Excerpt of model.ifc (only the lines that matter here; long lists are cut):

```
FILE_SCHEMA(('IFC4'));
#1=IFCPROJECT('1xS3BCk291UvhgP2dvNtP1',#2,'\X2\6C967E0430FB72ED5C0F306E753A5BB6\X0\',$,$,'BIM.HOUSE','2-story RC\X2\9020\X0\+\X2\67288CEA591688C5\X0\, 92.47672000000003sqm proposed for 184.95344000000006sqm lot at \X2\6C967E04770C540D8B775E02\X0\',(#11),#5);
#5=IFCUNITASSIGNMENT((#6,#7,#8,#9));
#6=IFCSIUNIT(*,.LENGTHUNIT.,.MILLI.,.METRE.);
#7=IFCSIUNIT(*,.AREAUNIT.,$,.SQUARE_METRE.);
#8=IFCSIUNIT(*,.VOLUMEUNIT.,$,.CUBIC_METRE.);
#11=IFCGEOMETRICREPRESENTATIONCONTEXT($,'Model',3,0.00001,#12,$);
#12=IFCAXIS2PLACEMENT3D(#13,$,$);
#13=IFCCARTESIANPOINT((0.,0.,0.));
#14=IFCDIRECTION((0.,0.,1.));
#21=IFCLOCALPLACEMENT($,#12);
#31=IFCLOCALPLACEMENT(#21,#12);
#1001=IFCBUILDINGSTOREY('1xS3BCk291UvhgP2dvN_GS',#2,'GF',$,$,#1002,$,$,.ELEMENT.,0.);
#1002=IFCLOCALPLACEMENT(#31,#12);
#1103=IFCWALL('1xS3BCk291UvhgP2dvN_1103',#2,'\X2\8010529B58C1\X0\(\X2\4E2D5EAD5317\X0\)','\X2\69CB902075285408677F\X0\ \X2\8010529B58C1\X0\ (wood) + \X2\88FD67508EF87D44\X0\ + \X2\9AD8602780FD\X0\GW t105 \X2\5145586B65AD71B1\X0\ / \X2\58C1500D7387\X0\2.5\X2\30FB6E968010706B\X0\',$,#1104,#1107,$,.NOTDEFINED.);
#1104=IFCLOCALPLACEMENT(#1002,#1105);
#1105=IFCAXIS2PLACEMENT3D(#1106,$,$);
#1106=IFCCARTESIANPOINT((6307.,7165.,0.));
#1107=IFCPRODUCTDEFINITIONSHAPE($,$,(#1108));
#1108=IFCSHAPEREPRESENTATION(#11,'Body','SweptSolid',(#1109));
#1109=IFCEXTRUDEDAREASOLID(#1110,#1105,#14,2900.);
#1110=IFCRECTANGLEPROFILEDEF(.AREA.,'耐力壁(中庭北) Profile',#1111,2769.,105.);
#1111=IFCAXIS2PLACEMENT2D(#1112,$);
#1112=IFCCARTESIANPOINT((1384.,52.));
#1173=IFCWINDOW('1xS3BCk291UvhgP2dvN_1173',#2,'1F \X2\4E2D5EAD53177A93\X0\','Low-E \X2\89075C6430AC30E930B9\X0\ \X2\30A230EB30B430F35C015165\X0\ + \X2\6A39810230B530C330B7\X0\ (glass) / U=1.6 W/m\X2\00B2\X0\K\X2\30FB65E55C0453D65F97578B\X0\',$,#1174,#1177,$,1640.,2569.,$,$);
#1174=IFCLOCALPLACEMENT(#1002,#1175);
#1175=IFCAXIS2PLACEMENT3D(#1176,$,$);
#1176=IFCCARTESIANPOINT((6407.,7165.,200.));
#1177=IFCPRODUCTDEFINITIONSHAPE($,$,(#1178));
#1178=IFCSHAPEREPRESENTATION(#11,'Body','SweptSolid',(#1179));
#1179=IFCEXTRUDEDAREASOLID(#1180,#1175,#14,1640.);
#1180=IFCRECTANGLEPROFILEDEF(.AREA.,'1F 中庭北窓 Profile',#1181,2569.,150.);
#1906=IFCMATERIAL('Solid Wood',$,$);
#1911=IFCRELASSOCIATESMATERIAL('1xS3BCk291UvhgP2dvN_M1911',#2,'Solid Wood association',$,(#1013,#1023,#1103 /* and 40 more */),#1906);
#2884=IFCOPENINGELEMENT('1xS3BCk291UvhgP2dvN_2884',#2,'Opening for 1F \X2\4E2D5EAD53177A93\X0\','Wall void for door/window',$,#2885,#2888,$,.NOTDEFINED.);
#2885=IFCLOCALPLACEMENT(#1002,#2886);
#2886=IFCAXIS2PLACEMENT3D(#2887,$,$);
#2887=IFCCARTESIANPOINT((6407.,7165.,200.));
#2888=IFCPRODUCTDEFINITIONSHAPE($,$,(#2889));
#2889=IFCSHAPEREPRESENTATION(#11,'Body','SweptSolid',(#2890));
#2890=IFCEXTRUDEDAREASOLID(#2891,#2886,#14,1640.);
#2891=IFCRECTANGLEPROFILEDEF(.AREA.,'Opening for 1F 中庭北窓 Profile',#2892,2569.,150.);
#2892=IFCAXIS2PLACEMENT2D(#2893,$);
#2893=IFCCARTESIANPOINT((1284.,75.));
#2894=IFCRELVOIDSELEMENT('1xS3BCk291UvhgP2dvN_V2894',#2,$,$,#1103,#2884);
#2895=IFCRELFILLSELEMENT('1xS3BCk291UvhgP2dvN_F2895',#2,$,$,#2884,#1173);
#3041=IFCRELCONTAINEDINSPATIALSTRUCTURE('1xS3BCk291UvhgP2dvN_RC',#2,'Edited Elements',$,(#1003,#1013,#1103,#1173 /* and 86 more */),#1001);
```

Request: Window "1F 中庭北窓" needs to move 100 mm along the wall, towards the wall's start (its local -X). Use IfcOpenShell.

```python
import ifcopenshell
import ifcopenshell.api.geometry
import ifcopenshell.util.placement

model = ifcopenshell.open("model.ifc")

window = model.by_guid("1xS3BCk291UvhgP2dvN_1173")
opening = window.FillsVoids[0].RelatingOpeningElement
wall = opening.VoidsElements[0].RelatingBuildingElement

wall_matrix = ifcopenshell.util.placement.get_local_placement(wall.ObjectPlacement)
shift = wall_matrix[:3, 0] * -100.0
before = ifcopenshell.util.placement.get_local_placement(window.ObjectPlacement)[:3, 3].copy()

# The window is not placed relative to its opening, so move both.
for product in (opening, window):
    matrix = ifcopenshell.util.placement.get_local_placement(product.ObjectPlacement)
    matrix[:3, 3] += shift
    ifcopenshell.api.geometry.edit_object_placement(model, product=product, matrix=matrix, is_si=False)

after = ifcopenshell.util.placement.get_local_placement(window.ObjectPlacement)[:3, 3]
print("window moved by", (after - before).round(3) + 0.0)

model.write("model_v2.ifc")
```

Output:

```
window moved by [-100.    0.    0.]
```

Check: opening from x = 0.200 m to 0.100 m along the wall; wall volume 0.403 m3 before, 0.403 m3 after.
